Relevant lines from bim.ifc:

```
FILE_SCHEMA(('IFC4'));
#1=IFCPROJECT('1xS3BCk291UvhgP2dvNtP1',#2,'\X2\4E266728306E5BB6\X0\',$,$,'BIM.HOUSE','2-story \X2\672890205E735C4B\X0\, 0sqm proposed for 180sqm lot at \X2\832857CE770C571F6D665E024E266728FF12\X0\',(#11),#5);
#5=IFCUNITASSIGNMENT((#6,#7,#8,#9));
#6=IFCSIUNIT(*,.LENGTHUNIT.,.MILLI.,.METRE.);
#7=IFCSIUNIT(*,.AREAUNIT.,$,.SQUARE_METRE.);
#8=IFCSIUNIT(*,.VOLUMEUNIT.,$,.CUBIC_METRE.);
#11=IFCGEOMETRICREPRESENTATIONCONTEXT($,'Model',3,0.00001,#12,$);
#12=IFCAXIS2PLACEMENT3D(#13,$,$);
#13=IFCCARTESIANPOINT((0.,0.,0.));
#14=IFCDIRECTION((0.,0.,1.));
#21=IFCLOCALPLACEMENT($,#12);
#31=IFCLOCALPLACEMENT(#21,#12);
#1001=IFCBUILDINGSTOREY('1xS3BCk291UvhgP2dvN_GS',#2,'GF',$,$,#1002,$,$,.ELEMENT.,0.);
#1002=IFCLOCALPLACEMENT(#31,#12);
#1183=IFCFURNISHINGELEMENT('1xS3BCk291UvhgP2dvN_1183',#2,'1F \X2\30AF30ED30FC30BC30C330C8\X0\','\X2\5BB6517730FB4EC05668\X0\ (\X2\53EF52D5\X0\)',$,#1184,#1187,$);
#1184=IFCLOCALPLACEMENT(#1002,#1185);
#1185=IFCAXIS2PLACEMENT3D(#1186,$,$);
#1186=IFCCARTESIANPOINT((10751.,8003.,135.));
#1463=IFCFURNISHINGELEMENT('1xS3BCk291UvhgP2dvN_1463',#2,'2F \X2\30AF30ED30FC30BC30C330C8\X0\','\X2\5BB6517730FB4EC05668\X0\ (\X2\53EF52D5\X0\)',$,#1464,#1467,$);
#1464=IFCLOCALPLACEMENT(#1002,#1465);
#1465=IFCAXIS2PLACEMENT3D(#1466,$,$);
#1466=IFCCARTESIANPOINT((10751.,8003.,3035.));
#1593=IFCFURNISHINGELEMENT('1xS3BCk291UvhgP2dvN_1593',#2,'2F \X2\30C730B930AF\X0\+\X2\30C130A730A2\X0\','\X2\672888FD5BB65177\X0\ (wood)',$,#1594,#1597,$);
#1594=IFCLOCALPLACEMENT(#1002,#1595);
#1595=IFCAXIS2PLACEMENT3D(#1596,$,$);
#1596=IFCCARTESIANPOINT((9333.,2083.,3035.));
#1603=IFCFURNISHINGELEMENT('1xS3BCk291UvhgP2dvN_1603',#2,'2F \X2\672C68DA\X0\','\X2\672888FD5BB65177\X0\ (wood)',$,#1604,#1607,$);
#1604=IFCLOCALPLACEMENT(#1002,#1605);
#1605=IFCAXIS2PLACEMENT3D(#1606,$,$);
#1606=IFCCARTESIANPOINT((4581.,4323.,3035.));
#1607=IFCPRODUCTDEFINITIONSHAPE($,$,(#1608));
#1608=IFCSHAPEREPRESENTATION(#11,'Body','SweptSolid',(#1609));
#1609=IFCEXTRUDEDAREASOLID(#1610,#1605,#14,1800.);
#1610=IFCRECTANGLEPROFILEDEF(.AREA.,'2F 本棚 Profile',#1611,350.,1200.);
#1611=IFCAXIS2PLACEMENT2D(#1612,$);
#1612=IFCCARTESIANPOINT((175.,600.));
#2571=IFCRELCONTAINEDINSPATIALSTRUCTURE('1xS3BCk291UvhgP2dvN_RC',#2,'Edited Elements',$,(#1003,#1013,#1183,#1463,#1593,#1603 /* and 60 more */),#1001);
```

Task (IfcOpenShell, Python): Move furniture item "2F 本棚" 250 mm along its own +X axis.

```python
import ifcopenshell
import ifcopenshell.api.geometry
import ifcopenshell.util.placement

model = ifcopenshell.open("bim.ifc")

item = model.by_guid("1xS3BCk291UvhgP2dvN_1603")
matrix = ifcopenshell.util.placement.get_local_placement(item.ObjectPlacement)
matrix[:3, 3] += matrix[:3, 0] * 250.0
ifcopenshell.api.geometry.edit_object_placement(model, product=item, matrix=matrix, is_si=False)

print(ifcopenshell.util.placement.get_local_placement(item.ObjectPlacement).round(3) + 0.0)

model.write("bim_v2.ifc")
```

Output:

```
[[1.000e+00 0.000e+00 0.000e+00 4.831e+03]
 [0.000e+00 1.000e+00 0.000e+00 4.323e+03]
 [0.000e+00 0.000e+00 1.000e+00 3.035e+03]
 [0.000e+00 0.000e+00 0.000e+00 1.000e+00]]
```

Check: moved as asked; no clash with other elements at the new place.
